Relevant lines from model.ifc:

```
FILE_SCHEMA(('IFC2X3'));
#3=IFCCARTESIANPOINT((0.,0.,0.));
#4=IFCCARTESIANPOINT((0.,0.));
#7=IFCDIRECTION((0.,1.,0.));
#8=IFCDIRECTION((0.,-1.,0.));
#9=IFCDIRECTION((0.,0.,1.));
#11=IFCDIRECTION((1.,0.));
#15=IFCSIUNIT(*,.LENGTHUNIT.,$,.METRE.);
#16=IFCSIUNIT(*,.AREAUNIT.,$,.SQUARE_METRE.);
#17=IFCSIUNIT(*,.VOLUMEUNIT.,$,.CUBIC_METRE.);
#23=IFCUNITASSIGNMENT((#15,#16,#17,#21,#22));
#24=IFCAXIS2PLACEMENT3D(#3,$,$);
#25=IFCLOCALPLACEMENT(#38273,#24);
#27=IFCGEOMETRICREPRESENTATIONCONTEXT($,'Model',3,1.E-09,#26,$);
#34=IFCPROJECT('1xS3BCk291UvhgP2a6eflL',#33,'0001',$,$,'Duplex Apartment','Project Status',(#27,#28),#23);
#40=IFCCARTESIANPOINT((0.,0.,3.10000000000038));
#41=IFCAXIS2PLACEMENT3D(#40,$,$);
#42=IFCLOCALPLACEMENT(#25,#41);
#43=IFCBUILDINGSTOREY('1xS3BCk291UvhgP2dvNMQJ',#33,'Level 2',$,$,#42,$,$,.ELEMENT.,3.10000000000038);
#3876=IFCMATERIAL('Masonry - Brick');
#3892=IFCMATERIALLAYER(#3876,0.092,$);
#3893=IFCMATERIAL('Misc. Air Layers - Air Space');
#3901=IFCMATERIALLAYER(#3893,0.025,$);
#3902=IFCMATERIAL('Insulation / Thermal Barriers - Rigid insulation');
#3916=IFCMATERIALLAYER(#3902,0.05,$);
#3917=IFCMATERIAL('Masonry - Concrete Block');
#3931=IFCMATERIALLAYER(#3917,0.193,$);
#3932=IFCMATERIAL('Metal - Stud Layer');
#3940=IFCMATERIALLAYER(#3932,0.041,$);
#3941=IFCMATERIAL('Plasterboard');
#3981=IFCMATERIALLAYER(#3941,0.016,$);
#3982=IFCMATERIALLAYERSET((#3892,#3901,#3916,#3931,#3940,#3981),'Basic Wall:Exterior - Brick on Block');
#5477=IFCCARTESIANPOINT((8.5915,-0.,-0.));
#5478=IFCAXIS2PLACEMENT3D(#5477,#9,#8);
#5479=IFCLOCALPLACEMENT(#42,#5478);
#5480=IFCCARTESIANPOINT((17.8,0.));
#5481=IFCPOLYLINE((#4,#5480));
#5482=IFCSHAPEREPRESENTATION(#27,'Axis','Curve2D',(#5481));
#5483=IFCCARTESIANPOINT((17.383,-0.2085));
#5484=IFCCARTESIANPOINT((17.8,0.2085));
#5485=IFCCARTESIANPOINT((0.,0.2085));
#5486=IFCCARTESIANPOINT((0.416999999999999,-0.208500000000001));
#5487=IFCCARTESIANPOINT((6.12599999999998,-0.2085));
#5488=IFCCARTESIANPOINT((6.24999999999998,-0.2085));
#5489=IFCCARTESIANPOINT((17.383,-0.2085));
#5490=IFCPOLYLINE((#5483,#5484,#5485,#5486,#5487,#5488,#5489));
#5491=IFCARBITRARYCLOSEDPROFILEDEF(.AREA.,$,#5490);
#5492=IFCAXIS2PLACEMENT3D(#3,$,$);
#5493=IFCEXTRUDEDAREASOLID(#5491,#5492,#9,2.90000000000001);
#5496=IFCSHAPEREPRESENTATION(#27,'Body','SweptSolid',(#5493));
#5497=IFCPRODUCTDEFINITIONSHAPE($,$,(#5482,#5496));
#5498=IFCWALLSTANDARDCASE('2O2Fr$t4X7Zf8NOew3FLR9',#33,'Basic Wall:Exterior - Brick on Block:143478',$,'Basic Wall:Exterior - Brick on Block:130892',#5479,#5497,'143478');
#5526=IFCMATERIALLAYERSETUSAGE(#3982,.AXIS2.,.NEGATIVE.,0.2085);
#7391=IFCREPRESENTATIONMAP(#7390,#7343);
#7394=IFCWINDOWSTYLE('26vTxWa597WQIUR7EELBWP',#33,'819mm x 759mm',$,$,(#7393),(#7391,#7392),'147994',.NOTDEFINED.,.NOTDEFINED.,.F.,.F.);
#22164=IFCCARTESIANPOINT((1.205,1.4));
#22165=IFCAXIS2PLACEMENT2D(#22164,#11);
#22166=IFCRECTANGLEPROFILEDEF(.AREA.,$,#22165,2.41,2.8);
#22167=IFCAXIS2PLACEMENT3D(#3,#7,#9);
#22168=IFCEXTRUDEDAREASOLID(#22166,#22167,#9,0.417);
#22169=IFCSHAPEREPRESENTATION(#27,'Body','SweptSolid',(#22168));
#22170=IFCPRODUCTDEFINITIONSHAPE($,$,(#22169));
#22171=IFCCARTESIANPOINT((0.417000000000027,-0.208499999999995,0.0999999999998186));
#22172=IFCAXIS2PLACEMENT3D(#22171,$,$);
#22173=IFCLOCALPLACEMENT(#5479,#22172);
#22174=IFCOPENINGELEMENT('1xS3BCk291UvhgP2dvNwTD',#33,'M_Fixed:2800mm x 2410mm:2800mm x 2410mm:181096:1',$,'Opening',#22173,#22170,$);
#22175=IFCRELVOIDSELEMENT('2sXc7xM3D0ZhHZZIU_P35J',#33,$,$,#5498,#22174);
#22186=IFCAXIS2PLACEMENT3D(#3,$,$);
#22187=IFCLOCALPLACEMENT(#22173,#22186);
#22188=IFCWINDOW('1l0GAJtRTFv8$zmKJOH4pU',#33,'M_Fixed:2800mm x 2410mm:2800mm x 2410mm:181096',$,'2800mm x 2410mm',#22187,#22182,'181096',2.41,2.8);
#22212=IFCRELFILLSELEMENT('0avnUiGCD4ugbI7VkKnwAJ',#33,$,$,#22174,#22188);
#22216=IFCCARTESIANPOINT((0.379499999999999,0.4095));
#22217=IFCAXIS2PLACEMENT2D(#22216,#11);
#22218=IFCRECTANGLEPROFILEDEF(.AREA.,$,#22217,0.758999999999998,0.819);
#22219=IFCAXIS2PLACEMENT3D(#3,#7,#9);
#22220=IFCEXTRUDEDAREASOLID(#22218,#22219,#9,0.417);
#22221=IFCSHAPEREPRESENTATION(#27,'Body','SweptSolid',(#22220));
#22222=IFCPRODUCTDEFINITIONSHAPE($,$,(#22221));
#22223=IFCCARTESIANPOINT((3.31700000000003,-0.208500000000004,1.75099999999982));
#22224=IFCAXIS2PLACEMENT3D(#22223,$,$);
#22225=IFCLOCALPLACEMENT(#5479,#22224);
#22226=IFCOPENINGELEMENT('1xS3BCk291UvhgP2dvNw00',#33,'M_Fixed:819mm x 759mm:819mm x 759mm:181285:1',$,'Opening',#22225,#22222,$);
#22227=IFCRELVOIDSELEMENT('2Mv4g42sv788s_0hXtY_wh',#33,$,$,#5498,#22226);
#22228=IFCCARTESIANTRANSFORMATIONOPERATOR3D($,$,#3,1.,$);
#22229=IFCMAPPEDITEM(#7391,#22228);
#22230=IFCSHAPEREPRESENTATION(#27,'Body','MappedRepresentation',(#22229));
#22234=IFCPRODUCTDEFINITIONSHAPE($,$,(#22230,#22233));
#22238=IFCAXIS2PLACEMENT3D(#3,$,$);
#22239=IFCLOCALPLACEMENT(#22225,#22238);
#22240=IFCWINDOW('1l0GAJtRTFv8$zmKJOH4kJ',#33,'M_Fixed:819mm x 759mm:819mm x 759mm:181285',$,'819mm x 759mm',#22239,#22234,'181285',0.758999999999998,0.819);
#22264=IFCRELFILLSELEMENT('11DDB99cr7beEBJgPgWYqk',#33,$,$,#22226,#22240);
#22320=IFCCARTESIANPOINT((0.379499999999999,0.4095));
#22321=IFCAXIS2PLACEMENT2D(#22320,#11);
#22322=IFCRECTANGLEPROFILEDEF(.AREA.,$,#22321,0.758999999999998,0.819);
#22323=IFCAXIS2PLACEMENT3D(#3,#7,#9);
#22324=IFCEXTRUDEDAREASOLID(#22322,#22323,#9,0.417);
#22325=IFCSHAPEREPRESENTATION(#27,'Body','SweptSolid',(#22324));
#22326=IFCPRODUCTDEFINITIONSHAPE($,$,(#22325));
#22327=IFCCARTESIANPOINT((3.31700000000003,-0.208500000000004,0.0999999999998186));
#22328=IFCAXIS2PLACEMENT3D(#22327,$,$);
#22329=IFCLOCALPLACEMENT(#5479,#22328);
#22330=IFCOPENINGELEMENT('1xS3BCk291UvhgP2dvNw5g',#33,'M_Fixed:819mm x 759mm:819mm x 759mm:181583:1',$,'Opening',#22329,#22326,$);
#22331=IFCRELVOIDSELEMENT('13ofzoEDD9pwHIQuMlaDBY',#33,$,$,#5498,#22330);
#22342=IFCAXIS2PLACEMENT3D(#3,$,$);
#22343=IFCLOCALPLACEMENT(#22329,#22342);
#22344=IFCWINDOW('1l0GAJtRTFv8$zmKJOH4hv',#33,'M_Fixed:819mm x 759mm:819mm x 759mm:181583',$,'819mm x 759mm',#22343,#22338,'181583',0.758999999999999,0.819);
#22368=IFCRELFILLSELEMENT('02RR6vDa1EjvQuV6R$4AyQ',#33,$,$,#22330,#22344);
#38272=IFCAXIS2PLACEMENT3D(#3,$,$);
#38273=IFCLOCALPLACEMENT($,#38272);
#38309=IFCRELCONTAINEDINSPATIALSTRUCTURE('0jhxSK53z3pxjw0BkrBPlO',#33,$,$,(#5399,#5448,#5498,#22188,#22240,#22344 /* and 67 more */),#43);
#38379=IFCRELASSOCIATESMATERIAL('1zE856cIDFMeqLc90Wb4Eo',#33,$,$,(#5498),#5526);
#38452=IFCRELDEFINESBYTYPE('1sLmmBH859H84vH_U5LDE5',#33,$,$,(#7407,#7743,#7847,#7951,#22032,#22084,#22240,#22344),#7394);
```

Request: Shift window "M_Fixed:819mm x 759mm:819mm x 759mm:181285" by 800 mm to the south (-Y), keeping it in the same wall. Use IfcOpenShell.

```python
import ifcopenshell
import ifcopenshell.api.geometry
import ifcopenshell.util.placement

model = ifcopenshell.open("model.ifc")

window = model.by_guid("1l0GAJtRTFv8$zmKJOH4kJ")
opening = window.FillsVoids[0].RelatingOpeningElement
wall = opening.VoidsElements[0].RelatingBuildingElement

wall_matrix = ifcopenshell.util.placement.get_local_placement(wall.ObjectPlacement)
shift = wall_matrix[:3, 0] * 0.8
before = ifcopenshell.util.placement.get_local_placement(window.ObjectPlacement)[:3, 3].copy()

# The window is placed relative to its opening, so it follows when the opening moves.
matrix = ifcopenshell.util.placement.get_local_placement(opening.ObjectPlacement)
matrix[:3, 3] += shift
ifcopenshell.api.geometry.edit_object_placement(
    model, product=opening, matrix=matrix, is_si=False, should_transform_children=True
)

after = ifcopenshell.util.placement.get_local_placement(window.ObjectPlacement)[:3, 3]
print("window moved by", (after - before).round(3) + 0.0)

model.write("model_edited.ifc")
```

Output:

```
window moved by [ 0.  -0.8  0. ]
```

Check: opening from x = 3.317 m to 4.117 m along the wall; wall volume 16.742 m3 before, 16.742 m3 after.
